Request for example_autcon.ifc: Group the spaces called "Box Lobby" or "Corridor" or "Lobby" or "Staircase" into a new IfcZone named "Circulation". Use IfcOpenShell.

First a look at what the model holds.

```python
import ifcopenshell

model = ifcopenshell.open("example_autcon.ifc")
print(model.schema)
seen = {}
for space in model.by_type("IfcSpace"):
    seen[space.LongName] = seen.get(space.LongName, 0) + 1
for name, count in sorted(seen.items(), key=str):
    print(count, "x", name)
print("zones:", [z.Name for z in model.by_type("IfcZone")][:20])
```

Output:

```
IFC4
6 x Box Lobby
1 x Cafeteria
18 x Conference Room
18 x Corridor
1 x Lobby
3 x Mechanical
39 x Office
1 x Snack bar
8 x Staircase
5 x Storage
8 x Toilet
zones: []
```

```python
import ifcopenshell
import ifcopenshell.api.group
import ifcopenshell.api.root

model = ifcopenshell.open("example_autcon.ifc")

names = {"Box Lobby", "Corridor", "Lobby", "Staircase"}
spaces = [s for s in model.by_type("IfcSpace") if s.LongName in names]

zone = ifcopenshell.api.root.create_entity(model, ifc_class="IfcZone", name="Circulation")
ifcopenshell.api.group.assign_group(model, products=spaces, group=zone)
print(len(spaces), "spaces in", zone.Name)

model.write("example_autcon_v2.ifc")
```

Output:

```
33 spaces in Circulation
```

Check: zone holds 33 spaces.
